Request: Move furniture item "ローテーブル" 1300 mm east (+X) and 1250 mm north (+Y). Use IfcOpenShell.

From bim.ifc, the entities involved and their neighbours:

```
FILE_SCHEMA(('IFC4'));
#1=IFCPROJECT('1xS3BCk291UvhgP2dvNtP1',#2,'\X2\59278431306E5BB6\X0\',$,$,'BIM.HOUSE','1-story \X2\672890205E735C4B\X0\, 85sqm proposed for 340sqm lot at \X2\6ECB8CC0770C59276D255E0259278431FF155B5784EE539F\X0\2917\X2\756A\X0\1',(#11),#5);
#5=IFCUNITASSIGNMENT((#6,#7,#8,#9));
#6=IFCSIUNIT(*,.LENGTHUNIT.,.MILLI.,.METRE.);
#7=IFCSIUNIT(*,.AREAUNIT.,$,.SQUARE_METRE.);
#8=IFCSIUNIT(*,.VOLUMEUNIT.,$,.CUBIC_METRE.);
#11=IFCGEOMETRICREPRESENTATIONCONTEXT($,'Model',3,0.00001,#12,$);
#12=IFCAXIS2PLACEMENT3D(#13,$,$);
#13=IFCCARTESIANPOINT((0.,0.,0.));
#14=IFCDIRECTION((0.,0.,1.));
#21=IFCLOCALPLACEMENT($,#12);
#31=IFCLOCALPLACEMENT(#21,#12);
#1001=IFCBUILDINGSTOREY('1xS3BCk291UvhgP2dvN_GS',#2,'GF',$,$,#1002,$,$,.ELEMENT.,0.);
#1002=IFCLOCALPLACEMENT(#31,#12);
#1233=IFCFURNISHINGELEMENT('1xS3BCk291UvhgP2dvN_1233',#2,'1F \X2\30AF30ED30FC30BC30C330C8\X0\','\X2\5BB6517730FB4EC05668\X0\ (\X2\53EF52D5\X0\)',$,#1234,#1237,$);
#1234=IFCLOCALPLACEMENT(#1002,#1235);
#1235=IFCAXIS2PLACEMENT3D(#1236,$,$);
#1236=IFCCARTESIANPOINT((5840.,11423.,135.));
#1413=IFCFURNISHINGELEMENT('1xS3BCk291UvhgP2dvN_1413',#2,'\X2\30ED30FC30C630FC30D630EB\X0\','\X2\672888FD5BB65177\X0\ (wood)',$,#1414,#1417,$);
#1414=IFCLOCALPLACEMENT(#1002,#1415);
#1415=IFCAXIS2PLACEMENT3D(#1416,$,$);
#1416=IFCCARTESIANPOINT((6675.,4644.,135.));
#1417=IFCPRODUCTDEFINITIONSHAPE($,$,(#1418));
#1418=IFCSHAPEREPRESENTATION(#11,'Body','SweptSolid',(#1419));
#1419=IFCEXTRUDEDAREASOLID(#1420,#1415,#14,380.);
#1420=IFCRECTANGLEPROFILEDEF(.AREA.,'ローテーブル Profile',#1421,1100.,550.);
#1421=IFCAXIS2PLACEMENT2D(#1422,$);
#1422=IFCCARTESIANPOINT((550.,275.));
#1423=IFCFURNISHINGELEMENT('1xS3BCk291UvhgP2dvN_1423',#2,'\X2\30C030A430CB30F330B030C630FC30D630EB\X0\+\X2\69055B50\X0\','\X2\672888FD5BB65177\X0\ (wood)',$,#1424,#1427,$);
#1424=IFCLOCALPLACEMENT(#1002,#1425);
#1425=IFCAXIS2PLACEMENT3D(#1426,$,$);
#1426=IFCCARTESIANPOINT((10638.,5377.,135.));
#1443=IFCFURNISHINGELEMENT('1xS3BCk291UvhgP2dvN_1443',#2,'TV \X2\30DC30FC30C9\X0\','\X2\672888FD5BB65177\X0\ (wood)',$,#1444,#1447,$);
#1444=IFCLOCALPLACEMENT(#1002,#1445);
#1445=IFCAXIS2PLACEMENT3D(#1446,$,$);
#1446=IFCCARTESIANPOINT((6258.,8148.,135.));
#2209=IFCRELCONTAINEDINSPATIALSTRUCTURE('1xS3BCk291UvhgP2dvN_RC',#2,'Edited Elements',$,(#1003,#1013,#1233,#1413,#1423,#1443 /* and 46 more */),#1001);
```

```python
import ifcopenshell
import ifcopenshell.api.geometry
import ifcopenshell.util.placement
import ifcopenshell.util.unit

model = ifcopenshell.open("bim.ifc")
unit_scale = ifcopenshell.util.unit.calculate_unit_scale(model)

item = model.by_guid("1xS3BCk291UvhgP2dvN_1413")
matrix = ifcopenshell.util.placement.get_local_placement(item.ObjectPlacement)
matrix[0, 3] += 1.3 / unit_scale
matrix[1, 3] += 1.25 / unit_scale
ifcopenshell.api.geometry.edit_object_placement(model, product=item, matrix=matrix, is_si=False)

print(ifcopenshell.util.placement.get_local_placement(item.ObjectPlacement).round(3) + 0.0)

model.write("bim_edited.ifc")
```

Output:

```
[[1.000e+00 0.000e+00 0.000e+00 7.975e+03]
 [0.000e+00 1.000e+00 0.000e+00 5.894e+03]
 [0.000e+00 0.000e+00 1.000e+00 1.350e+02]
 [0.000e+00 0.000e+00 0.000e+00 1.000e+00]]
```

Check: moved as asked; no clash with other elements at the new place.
